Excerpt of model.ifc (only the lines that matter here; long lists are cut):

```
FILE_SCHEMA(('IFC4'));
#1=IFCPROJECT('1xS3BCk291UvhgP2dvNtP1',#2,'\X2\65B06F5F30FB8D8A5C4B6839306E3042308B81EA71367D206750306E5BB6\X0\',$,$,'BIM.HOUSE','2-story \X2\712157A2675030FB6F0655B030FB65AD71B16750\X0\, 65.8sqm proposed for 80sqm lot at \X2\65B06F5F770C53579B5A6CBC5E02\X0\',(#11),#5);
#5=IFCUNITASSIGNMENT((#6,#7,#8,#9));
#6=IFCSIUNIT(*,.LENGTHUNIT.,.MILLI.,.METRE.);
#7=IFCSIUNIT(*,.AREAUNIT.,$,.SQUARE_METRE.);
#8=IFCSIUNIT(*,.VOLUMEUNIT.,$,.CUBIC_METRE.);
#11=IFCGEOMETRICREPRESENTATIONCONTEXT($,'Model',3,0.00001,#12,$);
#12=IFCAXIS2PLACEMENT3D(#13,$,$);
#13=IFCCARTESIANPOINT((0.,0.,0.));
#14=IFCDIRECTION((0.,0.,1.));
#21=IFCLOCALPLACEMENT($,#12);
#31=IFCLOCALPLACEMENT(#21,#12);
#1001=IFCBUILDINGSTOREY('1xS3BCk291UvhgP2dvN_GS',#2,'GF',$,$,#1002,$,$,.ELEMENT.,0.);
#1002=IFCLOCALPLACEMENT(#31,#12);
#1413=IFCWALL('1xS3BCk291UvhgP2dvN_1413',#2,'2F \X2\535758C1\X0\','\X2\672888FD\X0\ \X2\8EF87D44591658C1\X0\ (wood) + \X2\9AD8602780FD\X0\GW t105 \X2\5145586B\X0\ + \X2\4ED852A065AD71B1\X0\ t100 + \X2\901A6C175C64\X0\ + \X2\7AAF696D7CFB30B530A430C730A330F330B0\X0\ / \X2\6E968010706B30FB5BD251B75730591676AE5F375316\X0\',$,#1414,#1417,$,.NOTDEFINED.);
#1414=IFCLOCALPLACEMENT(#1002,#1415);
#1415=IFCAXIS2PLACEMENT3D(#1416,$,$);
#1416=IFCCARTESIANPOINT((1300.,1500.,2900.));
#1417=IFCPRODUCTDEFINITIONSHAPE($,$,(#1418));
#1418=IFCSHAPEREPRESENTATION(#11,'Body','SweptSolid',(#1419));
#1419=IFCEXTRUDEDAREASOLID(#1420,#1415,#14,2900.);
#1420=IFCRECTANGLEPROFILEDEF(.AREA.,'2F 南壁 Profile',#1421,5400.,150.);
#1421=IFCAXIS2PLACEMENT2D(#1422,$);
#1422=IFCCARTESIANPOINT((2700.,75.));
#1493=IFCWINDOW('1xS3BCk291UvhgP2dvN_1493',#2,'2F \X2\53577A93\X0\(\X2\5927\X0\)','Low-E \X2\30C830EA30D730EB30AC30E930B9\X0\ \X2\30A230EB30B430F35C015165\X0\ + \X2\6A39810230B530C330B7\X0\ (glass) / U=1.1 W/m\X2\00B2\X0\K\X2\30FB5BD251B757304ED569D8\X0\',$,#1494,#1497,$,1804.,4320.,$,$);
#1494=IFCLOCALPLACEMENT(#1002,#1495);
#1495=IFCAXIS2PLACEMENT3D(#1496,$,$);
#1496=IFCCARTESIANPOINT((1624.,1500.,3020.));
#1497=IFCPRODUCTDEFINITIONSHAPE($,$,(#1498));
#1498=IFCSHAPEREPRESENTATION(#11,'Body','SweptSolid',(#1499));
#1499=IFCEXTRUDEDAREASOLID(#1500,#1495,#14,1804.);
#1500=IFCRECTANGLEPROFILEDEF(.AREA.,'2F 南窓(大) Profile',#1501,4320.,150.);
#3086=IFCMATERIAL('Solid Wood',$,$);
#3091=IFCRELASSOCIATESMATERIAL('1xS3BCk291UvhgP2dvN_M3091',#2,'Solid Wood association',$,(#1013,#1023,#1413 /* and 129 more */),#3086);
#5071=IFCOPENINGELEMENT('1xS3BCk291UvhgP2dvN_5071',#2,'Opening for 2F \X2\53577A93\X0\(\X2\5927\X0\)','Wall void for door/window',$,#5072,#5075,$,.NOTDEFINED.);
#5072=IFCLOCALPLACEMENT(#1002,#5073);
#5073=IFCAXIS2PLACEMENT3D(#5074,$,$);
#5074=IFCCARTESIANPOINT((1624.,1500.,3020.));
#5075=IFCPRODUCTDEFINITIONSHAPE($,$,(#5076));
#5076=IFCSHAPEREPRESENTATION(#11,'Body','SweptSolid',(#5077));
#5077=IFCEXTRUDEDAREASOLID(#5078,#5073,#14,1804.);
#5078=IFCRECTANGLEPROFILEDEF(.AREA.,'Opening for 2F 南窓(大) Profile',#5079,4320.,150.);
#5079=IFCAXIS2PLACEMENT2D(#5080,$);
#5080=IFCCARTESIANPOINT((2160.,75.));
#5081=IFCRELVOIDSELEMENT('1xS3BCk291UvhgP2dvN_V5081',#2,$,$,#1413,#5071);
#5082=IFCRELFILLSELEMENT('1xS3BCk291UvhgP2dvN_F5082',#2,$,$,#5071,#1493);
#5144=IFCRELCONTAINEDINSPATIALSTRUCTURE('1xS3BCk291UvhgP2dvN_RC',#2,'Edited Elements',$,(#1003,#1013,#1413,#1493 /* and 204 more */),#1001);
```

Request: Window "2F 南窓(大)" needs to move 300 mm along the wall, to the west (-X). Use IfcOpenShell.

```python
import ifcopenshell
import ifcopenshell.api.geometry
import ifcopenshell.util.placement
import ifcopenshell.util.unit

model = ifcopenshell.open("model.ifc")
unit_scale = ifcopenshell.util.unit.calculate_unit_scale(model)

window = model.by_guid("1xS3BCk291UvhgP2dvN_1493")
opening = window.FillsVoids[0].RelatingOpeningElement
wall = opening.VoidsElements[0].RelatingBuildingElement

wall_matrix = ifcopenshell.util.placement.get_local_placement(wall.ObjectPlacement)
shift = wall_matrix[:3, 0] * -0.3 / unit_scale
before = ifcopenshell.util.placement.get_local_placement(window.ObjectPlacement)[:3, 3].copy()

# The window is not placed relative to its opening, so move both.
for product in (opening, window):
    matrix = ifcopenshell.util.placement.get_local_placement(product.ObjectPlacement)
    matrix[:3, 3] += shift
    ifcopenshell.api.geometry.edit_object_placement(model, product=product, matrix=matrix, is_si=False)

after = ifcopenshell.util.placement.get_local_placement(window.ObjectPlacement)[:3, 3]
print("window moved by", (after - before).round(3) + 0.0)

model.write("model_v2.ifc")
```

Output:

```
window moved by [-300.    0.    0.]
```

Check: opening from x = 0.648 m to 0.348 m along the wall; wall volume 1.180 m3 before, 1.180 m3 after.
